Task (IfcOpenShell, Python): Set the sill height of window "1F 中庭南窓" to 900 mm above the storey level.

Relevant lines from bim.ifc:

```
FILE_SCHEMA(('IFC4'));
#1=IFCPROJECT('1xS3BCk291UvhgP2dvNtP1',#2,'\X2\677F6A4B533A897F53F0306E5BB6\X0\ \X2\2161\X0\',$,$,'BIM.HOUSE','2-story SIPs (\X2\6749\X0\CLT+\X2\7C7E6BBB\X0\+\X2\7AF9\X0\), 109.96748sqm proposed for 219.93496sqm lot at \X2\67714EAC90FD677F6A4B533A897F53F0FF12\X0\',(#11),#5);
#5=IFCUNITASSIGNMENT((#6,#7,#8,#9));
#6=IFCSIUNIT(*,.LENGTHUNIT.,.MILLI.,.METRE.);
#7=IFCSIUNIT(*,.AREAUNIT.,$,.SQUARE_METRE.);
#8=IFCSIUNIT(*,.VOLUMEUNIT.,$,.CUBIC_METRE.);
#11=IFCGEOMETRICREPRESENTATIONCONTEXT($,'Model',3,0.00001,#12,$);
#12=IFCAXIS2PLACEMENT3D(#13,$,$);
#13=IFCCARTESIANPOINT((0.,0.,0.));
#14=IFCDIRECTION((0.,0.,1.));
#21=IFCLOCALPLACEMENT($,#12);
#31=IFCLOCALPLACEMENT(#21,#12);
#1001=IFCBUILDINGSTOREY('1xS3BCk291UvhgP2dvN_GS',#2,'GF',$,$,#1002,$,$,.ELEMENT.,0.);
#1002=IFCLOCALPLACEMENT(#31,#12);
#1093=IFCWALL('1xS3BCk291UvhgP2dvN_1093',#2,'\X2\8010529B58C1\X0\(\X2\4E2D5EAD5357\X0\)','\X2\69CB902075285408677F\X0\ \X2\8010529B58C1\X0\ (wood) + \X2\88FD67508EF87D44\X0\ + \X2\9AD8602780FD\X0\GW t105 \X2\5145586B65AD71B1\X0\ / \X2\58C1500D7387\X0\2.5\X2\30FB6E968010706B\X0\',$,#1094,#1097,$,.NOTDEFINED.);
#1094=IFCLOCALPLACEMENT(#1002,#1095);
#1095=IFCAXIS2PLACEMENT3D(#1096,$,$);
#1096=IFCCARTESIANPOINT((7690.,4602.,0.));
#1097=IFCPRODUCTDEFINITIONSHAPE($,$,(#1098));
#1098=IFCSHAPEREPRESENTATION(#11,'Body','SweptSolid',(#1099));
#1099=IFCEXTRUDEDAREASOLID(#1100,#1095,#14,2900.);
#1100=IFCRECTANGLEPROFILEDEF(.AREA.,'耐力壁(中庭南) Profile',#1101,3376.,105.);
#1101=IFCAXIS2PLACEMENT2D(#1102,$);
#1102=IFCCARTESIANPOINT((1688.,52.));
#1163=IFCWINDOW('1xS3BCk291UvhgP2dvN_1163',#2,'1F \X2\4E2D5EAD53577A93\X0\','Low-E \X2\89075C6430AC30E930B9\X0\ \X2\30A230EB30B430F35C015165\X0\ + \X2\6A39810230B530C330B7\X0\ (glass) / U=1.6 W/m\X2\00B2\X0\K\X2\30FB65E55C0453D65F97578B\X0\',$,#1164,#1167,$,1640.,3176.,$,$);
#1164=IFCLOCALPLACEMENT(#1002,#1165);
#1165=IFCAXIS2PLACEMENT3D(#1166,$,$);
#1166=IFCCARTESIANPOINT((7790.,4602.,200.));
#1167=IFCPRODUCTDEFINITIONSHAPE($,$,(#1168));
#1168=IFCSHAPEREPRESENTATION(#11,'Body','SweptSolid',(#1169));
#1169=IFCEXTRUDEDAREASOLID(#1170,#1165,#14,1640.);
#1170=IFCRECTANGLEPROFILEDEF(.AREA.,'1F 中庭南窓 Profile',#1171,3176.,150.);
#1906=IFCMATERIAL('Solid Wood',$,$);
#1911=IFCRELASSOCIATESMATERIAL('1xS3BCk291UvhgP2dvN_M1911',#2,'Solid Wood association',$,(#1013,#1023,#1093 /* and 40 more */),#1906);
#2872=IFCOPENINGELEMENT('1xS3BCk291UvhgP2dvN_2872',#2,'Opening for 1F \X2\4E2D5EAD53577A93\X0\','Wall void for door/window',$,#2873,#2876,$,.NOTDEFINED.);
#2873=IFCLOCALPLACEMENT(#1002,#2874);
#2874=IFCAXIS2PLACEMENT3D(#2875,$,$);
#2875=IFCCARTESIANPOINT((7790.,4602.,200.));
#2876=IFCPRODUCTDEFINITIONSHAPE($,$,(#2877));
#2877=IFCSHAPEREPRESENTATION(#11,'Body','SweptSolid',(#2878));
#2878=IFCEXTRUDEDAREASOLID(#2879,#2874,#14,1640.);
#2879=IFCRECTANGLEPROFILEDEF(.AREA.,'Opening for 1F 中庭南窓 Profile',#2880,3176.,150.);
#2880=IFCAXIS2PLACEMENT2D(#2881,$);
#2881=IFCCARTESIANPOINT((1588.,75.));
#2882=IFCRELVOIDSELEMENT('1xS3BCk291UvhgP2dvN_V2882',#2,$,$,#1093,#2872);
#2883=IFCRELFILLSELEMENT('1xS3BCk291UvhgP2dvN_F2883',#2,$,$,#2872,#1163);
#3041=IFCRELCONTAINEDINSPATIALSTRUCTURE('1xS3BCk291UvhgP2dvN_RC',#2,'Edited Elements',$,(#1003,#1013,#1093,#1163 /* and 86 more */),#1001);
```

```python
import numpy as np
import ifcopenshell
import ifcopenshell.api.geometry
import ifcopenshell.geom
import ifcopenshell.util.element
import ifcopenshell.util.placement
import ifcopenshell.util.shape
import ifcopenshell.util.unit

model = ifcopenshell.open("bim.ifc")
unit_scale = ifcopenshell.util.unit.calculate_unit_scale(model)

window = model.by_guid("1xS3BCk291UvhgP2dvN_1163")
opening = window.FillsVoids[0].RelatingOpeningElement
storey = ifcopenshell.util.element.get_container(window, ifc_class="IfcBuildingStorey")
level = ifcopenshell.util.placement.get_local_placement(storey.ObjectPlacement)[2, 3]

# The opening's origin need not be at the sill, so measure its lowest point.
shape = ifcopenshell.geom.create_shape(ifcopenshell.geom.settings(), opening)
bottom = ifcopenshell.util.shape.get_shape_bottom_elevation(shape, shape.geometry) / unit_scale
dz = level + 900.0 - bottom

shift = np.array([0.0, 0.0, dz])
# The window is not placed relative to its opening, so move both.
for product in (opening, window):
    matrix = ifcopenshell.util.placement.get_local_placement(product.ObjectPlacement)
    matrix[:3, 3] += shift
    ifcopenshell.api.geometry.edit_object_placement(model, product=product, matrix=matrix, is_si=False)

print(f"moved by {dz * unit_scale:+.3f} m")

model.write("bim_edited.ifc")
```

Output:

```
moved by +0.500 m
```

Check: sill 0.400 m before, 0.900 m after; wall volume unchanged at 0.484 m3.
